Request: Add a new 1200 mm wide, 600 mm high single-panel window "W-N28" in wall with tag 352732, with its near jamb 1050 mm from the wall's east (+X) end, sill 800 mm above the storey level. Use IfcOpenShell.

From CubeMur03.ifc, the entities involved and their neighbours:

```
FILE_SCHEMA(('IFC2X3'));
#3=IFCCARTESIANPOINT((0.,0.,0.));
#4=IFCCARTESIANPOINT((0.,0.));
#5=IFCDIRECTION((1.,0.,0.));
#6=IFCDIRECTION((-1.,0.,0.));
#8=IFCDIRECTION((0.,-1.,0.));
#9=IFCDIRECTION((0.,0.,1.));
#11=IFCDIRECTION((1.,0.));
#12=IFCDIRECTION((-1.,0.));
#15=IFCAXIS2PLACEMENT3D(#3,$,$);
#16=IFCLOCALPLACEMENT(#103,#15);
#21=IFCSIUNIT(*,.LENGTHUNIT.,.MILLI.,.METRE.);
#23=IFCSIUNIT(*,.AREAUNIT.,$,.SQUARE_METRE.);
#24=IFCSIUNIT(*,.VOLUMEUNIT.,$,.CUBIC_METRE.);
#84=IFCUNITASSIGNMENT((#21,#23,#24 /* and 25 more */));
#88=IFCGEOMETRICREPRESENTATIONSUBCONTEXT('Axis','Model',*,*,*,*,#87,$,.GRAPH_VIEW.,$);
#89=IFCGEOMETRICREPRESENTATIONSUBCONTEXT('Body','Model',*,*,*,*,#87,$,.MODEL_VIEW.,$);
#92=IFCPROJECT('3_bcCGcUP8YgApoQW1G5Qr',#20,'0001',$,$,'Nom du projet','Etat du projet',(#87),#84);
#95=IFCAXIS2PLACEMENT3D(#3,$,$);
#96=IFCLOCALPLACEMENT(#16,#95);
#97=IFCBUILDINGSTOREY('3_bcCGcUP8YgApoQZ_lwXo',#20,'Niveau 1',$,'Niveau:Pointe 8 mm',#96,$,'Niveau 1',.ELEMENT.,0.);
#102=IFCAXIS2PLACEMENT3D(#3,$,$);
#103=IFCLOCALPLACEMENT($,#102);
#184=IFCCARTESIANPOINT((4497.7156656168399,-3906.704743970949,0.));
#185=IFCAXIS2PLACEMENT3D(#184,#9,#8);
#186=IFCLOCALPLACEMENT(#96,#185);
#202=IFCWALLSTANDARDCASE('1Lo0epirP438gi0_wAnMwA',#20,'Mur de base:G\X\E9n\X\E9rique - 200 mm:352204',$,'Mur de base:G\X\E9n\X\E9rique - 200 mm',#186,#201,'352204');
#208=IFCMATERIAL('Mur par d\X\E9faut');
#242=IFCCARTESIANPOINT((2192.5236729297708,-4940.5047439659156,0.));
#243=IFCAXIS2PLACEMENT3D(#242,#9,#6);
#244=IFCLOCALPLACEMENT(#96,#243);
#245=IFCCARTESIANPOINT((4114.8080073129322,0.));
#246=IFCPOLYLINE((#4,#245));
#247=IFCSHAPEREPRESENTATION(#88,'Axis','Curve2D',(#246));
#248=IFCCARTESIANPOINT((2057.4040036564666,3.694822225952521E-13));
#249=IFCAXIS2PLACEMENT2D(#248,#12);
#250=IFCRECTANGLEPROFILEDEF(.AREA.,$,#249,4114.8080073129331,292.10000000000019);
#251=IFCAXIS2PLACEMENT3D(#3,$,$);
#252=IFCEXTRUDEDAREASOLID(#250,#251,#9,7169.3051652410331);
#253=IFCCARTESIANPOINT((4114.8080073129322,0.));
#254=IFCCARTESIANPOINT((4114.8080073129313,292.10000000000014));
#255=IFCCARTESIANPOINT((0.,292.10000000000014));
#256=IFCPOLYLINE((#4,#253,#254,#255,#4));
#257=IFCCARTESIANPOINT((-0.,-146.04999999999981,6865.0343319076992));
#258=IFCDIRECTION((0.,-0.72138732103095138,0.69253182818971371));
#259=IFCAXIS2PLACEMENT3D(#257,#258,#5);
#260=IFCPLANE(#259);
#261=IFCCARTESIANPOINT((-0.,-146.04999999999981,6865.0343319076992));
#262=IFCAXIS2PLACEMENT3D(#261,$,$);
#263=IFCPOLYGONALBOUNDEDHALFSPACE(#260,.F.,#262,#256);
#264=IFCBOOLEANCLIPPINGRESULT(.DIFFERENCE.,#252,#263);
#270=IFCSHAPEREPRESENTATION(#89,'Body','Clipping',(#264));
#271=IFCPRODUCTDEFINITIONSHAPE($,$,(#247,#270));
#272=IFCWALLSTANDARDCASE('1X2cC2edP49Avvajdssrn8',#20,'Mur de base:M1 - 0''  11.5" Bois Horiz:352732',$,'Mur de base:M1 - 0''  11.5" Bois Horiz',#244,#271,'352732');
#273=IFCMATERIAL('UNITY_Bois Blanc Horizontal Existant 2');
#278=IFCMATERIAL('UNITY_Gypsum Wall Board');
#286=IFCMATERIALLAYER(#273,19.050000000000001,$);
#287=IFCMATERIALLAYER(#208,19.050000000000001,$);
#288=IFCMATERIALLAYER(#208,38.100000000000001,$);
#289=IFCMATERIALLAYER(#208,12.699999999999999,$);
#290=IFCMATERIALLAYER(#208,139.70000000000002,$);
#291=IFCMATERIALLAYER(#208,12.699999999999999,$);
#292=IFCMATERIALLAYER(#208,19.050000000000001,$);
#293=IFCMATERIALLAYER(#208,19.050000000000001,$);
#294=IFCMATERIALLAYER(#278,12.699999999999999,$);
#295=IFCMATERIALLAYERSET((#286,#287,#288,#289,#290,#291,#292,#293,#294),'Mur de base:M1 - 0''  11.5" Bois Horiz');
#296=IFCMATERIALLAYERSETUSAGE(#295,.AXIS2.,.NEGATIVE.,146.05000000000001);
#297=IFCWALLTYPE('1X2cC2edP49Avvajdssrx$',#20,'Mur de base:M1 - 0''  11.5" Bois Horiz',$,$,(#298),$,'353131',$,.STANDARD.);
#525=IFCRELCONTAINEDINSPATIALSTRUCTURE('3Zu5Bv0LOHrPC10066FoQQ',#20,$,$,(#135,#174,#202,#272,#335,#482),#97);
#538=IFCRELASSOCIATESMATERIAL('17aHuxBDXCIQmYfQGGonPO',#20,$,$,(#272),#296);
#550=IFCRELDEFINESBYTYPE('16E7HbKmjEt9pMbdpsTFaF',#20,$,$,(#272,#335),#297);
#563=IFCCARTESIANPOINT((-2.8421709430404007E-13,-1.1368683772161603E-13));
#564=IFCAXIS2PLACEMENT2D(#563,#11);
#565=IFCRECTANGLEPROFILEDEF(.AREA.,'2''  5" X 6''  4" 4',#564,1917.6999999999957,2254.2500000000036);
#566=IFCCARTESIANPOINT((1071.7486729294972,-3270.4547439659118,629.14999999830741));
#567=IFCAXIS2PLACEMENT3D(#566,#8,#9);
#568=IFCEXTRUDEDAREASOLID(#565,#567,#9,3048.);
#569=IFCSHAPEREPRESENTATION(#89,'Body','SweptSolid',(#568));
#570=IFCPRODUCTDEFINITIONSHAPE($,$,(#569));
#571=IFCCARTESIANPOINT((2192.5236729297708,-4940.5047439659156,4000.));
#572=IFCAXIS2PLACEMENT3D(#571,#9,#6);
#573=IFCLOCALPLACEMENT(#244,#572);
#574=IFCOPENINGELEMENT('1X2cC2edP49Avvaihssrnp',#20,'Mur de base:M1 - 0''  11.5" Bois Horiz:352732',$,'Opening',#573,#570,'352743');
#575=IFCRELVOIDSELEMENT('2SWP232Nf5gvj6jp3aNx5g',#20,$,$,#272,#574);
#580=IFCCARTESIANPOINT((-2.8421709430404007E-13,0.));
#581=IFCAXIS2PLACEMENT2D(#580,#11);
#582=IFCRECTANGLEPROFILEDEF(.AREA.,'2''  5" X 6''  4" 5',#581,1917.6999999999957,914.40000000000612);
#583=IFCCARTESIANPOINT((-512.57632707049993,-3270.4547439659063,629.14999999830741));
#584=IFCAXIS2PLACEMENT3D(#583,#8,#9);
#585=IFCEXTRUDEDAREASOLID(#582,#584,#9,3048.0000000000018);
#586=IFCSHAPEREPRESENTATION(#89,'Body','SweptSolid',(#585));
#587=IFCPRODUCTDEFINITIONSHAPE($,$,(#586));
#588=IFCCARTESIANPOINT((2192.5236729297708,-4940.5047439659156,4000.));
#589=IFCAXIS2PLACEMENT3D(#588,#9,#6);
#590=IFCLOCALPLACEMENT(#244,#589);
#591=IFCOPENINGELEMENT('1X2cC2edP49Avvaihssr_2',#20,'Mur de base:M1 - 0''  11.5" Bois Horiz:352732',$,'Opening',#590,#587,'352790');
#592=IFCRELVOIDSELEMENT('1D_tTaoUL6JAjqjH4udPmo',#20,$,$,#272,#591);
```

```python
import numpy as np
import ifcopenshell
import ifcopenshell.api.feature
import ifcopenshell.api.geometry
import ifcopenshell.api.root
import ifcopenshell.api.spatial
import ifcopenshell.api.type
import ifcopenshell.geom
import ifcopenshell.util.element
import ifcopenshell.util.placement
import ifcopenshell.util.representation
import ifcopenshell.util.shape
import ifcopenshell.util.unit

model = ifcopenshell.open("CubeMur03.ifc")
unit_scale = ifcopenshell.util.unit.calculate_unit_scale(model)
settings = ifcopenshell.geom.settings()


def volume(element):
    """Net volume in cubic metres, openings subtracted."""
    shape = ifcopenshell.geom.create_shape(settings, element)
    return ifcopenshell.util.shape.get_volume(shape.geometry)


wall = model.by_guid("1X2cC2edP49Avvajdssrn8")
storey = ifcopenshell.util.element.get_container(wall, ifc_class="IfcBuildingStorey")
context = ifcopenshell.util.representation.get_context(model, "Model", "Body", "MODEL_VIEW")
before = volume(wall)

width, height, from_end, sill = 1.2, 0.6, 1.05, 0.8  # metres

# The wall runs along its own X axis, and the end named is its -X end.
wall_shape = ifcopenshell.geom.create_shape(settings, wall)
x, y, z = ifcopenshell.util.shape.get_vertices(wall_shape.geometry).T
start = x.min() + from_end
face, thickness = float(y.min()), float(y.max() - y.min())
wall_matrix = ifcopenshell.util.placement.get_local_placement(wall.ObjectPlacement)
level = ifcopenshell.util.placement.get_local_placement(storey.ObjectPlacement)[2, 3]


def in_wall(x, y):
    """Placement at x, y metres in the wall's axes, at sill height."""
    matrix = wall_matrix.copy()
    matrix[:, 3] = wall_matrix @ np.array([x / unit_scale, y / unit_scale, 0.0, 1.0])
    matrix[2, 3] = level + sill / unit_scale
    return matrix


# Opening: a box that overshoots both wall faces by 50 mm.
opening = ifcopenshell.api.root.create_entity(model, ifc_class="IfcOpeningElement")
box = ifcopenshell.api.geometry.add_wall_representation(
    model, context=context, length=width, height=height, thickness=thickness + 0.1
)
ifcopenshell.api.geometry.assign_representation(model, product=opening, representation=box)
ifcopenshell.api.geometry.edit_object_placement(model, product=opening, matrix=in_wall(start, face - 0.05), is_si=False)
ifcopenshell.api.feature.add_feature(model, feature=opening, element=wall)

window = ifcopenshell.api.root.create_entity(model, ifc_class="IfcWindow", name="W-N28")
window.OverallWidth, window.OverallHeight = width / unit_scale, height / unit_scale
body = ifcopenshell.api.geometry.add_window_representation(
    model,
    context=context,
    overall_width=window.OverallWidth,
    overall_height=window.OverallHeight,
    partition_type="SINGLE_PANEL",
)
ifcopenshell.api.geometry.assign_representation(model, product=window, representation=body)
ifcopenshell.api.spatial.assign_container(model, products=[window], relating_structure=storey)
fills = ifcopenshell.api.feature.add_filling(model, opening=opening, element=window)
fills.OwnerHistory = window.OwnerHistory  # required in IFC2X3

# IFC2X3 keeps the operation on the window style.
style = ifcopenshell.api.root.create_entity(model, ifc_class="IfcWindowStyle", name="W-N28")
style.OperationType, style.ConstructionType = "SINGLE_PANEL", "NOTDEFINED"
style.ParameterTakesPrecedence = style.Sizeable = False
ifcopenshell.api.type.assign_type(model, related_objects=[window], relating_type=style)

# Centre the window in the wall's thickness.
ifcopenshell.api.geometry.edit_object_placement(model, product=window, matrix=in_wall(start, face), is_si=False)
window_shape = ifcopenshell.geom.create_shape(settings, window)
depth = ifcopenshell.util.shape.get_vertices(window_shape.geometry)[:, 1]
offset = face + thickness / 2 - (depth.min() + depth.max()) / 2
ifcopenshell.api.geometry.edit_object_placement(model, product=window, matrix=in_wall(start, offset), is_si=False)

after = volume(wall)

print(f"wall volume {before:.3f} -> {after:.3f} m3")

model.write("CubeMur03_edited.ifc")
```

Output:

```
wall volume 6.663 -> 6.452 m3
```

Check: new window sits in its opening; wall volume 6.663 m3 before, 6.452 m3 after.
